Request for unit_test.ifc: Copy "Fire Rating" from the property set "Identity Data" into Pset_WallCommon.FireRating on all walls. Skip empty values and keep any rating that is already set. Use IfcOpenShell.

First a look at what the model holds.

```python
import ifcopenshell
import ifcopenshell.util.element

model = ifcopenshell.open("unit_test.ifc")
print(model.schema)
walls = model.by_type("IfcWall")
print(len(walls), "walls")
for e in walls[:8]:
    source = ifcopenshell.util.element.get_pset(e, "Identity Data", "Fire Rating")
    target = ifcopenshell.util.element.get_pset(e, "Pset_WallCommon", "FireRating")
    print(e.id(), repr(source), repr(target), sep=" | ")
```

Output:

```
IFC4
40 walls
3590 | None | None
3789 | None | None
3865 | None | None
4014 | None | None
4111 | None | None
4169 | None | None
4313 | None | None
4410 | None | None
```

```python
import ifcopenshell
import ifcopenshell.api.pset
import ifcopenshell.util.element

model = ifcopenshell.open("unit_test.ifc")

count = 0
for e in model.by_type("IfcWall"):
    value = ifcopenshell.util.element.get_pset(e, "Identity Data", "Fire Rating")
    current = ifcopenshell.util.element.get_pset(e, "Pset_WallCommon", "FireRating")
    if not value or not value.strip() or current:
        continue
    # add_pset returns the element's existing set when there is one.
    pset = ifcopenshell.api.pset.add_pset(model, product=e, name="Pset_WallCommon")
    ifcopenshell.api.pset.edit_pset(model, pset=pset, properties={"FireRating": value})
    count += 1

print(count, "walls updated")

model.write("unit_test-out.ifc")
```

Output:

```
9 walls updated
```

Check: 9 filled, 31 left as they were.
